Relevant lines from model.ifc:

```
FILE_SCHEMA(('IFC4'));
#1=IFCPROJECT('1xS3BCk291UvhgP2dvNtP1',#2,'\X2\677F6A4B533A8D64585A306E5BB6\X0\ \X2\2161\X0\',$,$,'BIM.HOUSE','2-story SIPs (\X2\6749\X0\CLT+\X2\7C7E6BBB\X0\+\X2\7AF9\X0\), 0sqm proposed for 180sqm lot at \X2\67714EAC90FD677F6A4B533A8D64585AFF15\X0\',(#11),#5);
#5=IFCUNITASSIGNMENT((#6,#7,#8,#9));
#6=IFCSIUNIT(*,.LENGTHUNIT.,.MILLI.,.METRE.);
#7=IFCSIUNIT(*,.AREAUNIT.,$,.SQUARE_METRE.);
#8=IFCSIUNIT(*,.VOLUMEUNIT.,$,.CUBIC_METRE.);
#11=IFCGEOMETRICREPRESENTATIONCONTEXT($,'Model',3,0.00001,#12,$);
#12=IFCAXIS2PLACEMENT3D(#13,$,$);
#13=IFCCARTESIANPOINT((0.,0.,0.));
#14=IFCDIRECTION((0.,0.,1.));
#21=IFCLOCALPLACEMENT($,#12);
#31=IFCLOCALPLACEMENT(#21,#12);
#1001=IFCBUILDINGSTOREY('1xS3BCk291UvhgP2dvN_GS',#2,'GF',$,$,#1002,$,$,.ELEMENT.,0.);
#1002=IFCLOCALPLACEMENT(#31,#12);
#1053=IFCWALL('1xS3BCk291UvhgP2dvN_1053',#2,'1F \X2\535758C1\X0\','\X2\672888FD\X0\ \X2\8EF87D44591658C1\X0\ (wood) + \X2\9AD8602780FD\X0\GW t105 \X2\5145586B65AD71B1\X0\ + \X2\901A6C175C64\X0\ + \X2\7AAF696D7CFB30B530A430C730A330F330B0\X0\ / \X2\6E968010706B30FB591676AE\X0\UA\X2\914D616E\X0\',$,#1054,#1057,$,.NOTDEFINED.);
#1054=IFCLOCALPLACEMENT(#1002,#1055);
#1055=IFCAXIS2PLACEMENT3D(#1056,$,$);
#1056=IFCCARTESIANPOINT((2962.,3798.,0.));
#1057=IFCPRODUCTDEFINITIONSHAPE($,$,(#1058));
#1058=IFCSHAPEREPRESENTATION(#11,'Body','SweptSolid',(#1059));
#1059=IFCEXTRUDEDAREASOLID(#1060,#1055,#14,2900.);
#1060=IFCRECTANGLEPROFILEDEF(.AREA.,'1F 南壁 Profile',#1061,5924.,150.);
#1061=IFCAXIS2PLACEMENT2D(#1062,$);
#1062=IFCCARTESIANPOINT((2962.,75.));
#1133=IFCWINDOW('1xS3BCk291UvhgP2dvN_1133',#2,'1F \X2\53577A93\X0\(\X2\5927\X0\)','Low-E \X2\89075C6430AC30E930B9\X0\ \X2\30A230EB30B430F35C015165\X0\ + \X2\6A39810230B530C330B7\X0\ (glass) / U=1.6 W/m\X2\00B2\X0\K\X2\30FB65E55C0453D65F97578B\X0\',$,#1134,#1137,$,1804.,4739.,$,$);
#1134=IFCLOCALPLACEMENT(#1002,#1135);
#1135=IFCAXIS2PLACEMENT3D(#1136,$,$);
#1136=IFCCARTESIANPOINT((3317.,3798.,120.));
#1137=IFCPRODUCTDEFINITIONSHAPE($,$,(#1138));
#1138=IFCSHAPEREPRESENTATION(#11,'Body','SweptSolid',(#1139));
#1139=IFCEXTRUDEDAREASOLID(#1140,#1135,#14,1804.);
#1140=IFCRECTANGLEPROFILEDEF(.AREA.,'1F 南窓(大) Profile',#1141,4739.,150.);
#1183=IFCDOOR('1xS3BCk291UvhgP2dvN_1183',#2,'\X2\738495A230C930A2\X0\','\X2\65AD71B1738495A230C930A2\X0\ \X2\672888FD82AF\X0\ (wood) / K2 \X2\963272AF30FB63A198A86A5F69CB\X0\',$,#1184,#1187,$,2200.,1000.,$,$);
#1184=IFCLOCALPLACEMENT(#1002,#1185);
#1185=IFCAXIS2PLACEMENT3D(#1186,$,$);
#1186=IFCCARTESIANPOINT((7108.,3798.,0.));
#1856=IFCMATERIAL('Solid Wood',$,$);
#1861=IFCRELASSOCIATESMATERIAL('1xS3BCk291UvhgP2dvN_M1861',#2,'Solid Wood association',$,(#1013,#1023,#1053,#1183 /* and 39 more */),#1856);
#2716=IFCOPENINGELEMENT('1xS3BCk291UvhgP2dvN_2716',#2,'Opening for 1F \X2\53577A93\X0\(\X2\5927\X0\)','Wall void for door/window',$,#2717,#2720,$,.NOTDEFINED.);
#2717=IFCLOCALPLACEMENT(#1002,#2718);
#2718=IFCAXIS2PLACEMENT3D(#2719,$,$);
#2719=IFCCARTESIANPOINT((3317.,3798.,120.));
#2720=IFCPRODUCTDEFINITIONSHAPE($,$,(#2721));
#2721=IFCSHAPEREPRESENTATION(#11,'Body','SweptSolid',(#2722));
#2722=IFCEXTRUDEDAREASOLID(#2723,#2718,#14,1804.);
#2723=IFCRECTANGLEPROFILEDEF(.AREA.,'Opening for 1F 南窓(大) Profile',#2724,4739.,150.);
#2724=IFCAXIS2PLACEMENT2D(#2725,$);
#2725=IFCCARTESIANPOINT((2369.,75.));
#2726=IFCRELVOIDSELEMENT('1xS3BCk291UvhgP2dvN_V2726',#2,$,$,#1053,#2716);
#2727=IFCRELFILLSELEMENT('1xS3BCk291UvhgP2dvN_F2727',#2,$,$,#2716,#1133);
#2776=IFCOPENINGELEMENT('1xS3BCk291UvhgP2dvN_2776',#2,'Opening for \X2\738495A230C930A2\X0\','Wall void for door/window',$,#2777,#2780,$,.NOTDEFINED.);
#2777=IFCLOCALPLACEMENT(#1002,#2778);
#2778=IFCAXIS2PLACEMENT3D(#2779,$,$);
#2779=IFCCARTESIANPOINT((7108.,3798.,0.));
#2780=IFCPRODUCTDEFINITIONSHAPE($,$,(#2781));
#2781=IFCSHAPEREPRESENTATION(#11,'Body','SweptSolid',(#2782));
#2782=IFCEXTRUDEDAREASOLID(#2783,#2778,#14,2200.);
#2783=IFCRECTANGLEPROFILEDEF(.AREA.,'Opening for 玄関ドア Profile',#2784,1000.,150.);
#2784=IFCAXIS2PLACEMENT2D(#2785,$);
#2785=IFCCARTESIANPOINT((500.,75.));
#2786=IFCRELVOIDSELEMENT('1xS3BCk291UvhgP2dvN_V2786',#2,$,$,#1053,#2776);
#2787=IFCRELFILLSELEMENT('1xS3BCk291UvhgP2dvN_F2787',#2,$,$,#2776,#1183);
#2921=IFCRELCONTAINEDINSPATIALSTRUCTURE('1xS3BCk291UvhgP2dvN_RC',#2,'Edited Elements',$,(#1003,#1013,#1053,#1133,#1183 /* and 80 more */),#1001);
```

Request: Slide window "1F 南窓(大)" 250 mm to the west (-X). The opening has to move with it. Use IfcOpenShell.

```python
import ifcopenshell
import ifcopenshell.api.geometry
import ifcopenshell.util.placement
import ifcopenshell.util.unit

model = ifcopenshell.open("model.ifc")
unit_scale = ifcopenshell.util.unit.calculate_unit_scale(model)

window = model.by_guid("1xS3BCk291UvhgP2dvN_1133")
opening = window.FillsVoids[0].RelatingOpeningElement
wall = opening.VoidsElements[0].RelatingBuildingElement

wall_matrix = ifcopenshell.util.placement.get_local_placement(wall.ObjectPlacement)
shift = wall_matrix[:3, 0] * -0.25 / unit_scale
before = ifcopenshell.util.placement.get_local_placement(window.ObjectPlacement)[:3, 3].copy()

# The window is not placed relative to its opening, so move both.
for product in (opening, window):
    matrix = ifcopenshell.util.placement.get_local_placement(product.ObjectPlacement)
    matrix[:3, 3] += shift
    ifcopenshell.api.geometry.edit_object_placement(model, product=product, matrix=matrix, is_si=False)

after = ifcopenshell.util.placement.get_local_placement(window.ObjectPlacement)[:3, 3]
print("window moved by", (after - before).round(3) + 0.0)

model.write("model_edited.ifc")
```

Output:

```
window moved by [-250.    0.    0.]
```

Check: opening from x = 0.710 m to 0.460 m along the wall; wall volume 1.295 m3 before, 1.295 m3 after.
